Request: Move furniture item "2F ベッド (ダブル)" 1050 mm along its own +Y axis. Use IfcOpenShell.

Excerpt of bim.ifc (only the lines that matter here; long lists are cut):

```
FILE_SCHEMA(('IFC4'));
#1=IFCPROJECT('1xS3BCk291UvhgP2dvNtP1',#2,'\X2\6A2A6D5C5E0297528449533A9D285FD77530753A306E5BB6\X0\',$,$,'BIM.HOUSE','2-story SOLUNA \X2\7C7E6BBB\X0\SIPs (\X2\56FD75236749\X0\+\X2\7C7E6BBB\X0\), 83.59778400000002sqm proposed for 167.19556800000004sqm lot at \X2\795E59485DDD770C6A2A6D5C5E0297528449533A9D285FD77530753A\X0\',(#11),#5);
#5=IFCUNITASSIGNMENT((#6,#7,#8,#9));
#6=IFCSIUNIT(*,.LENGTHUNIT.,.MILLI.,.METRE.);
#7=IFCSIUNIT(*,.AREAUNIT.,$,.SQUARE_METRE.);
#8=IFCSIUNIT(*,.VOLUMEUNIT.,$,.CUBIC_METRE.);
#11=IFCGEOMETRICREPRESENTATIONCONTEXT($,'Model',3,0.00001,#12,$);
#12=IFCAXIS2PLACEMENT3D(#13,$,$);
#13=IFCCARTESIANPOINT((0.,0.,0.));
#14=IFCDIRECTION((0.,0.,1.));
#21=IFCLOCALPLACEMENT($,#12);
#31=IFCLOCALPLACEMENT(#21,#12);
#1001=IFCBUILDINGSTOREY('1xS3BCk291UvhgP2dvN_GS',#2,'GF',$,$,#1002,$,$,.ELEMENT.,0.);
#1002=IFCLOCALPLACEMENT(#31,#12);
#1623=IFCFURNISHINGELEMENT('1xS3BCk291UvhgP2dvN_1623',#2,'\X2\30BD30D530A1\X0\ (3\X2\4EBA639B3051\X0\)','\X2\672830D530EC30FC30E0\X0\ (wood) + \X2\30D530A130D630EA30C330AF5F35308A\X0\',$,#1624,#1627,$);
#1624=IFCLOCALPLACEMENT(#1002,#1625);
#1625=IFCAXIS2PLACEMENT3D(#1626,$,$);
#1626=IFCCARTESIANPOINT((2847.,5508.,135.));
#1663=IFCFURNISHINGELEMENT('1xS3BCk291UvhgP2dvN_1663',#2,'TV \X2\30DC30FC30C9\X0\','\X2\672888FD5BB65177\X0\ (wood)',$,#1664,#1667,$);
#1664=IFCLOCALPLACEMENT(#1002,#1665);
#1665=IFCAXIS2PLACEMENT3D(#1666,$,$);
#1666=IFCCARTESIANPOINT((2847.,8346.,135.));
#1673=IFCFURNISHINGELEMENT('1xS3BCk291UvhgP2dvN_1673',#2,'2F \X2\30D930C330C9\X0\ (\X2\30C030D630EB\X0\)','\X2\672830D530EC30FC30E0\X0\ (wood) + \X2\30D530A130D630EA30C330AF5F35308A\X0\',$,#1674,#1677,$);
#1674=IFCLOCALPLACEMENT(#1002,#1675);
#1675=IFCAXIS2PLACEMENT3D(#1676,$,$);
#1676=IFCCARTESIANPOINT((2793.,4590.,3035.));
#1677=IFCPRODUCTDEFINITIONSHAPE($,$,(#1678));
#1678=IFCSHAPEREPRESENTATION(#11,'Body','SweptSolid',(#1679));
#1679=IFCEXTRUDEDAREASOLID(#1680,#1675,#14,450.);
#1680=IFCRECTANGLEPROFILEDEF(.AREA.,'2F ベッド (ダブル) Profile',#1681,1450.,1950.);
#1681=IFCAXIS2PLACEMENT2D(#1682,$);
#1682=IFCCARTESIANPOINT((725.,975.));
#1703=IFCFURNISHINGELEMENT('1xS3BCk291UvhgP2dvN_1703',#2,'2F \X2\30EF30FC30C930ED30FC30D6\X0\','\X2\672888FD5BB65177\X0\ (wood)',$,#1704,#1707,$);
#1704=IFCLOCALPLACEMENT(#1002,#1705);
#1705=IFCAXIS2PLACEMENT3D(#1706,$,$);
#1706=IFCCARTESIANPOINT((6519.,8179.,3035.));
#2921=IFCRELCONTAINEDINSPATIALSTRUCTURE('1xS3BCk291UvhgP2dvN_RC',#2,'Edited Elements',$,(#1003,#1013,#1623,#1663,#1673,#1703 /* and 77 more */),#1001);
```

```python
import ifcopenshell
import ifcopenshell.api.geometry
import ifcopenshell.util.placement
import ifcopenshell.util.unit

model = ifcopenshell.open("bim.ifc")
unit_scale = ifcopenshell.util.unit.calculate_unit_scale(model)

item = model.by_guid("1xS3BCk291UvhgP2dvN_1673")
matrix = ifcopenshell.util.placement.get_local_placement(item.ObjectPlacement)
matrix[:3, 3] += matrix[:3, 1] * 1.05 / unit_scale
ifcopenshell.api.geometry.edit_object_placement(model, product=item, matrix=matrix, is_si=False)

print(ifcopenshell.util.placement.get_local_placement(item.ObjectPlacement).round(3) + 0.0)

model.write("bim_edited.ifc")
```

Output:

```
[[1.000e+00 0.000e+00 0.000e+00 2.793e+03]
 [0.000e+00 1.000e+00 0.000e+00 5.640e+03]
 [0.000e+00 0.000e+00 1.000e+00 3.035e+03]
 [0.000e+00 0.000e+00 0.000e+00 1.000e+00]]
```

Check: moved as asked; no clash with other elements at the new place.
